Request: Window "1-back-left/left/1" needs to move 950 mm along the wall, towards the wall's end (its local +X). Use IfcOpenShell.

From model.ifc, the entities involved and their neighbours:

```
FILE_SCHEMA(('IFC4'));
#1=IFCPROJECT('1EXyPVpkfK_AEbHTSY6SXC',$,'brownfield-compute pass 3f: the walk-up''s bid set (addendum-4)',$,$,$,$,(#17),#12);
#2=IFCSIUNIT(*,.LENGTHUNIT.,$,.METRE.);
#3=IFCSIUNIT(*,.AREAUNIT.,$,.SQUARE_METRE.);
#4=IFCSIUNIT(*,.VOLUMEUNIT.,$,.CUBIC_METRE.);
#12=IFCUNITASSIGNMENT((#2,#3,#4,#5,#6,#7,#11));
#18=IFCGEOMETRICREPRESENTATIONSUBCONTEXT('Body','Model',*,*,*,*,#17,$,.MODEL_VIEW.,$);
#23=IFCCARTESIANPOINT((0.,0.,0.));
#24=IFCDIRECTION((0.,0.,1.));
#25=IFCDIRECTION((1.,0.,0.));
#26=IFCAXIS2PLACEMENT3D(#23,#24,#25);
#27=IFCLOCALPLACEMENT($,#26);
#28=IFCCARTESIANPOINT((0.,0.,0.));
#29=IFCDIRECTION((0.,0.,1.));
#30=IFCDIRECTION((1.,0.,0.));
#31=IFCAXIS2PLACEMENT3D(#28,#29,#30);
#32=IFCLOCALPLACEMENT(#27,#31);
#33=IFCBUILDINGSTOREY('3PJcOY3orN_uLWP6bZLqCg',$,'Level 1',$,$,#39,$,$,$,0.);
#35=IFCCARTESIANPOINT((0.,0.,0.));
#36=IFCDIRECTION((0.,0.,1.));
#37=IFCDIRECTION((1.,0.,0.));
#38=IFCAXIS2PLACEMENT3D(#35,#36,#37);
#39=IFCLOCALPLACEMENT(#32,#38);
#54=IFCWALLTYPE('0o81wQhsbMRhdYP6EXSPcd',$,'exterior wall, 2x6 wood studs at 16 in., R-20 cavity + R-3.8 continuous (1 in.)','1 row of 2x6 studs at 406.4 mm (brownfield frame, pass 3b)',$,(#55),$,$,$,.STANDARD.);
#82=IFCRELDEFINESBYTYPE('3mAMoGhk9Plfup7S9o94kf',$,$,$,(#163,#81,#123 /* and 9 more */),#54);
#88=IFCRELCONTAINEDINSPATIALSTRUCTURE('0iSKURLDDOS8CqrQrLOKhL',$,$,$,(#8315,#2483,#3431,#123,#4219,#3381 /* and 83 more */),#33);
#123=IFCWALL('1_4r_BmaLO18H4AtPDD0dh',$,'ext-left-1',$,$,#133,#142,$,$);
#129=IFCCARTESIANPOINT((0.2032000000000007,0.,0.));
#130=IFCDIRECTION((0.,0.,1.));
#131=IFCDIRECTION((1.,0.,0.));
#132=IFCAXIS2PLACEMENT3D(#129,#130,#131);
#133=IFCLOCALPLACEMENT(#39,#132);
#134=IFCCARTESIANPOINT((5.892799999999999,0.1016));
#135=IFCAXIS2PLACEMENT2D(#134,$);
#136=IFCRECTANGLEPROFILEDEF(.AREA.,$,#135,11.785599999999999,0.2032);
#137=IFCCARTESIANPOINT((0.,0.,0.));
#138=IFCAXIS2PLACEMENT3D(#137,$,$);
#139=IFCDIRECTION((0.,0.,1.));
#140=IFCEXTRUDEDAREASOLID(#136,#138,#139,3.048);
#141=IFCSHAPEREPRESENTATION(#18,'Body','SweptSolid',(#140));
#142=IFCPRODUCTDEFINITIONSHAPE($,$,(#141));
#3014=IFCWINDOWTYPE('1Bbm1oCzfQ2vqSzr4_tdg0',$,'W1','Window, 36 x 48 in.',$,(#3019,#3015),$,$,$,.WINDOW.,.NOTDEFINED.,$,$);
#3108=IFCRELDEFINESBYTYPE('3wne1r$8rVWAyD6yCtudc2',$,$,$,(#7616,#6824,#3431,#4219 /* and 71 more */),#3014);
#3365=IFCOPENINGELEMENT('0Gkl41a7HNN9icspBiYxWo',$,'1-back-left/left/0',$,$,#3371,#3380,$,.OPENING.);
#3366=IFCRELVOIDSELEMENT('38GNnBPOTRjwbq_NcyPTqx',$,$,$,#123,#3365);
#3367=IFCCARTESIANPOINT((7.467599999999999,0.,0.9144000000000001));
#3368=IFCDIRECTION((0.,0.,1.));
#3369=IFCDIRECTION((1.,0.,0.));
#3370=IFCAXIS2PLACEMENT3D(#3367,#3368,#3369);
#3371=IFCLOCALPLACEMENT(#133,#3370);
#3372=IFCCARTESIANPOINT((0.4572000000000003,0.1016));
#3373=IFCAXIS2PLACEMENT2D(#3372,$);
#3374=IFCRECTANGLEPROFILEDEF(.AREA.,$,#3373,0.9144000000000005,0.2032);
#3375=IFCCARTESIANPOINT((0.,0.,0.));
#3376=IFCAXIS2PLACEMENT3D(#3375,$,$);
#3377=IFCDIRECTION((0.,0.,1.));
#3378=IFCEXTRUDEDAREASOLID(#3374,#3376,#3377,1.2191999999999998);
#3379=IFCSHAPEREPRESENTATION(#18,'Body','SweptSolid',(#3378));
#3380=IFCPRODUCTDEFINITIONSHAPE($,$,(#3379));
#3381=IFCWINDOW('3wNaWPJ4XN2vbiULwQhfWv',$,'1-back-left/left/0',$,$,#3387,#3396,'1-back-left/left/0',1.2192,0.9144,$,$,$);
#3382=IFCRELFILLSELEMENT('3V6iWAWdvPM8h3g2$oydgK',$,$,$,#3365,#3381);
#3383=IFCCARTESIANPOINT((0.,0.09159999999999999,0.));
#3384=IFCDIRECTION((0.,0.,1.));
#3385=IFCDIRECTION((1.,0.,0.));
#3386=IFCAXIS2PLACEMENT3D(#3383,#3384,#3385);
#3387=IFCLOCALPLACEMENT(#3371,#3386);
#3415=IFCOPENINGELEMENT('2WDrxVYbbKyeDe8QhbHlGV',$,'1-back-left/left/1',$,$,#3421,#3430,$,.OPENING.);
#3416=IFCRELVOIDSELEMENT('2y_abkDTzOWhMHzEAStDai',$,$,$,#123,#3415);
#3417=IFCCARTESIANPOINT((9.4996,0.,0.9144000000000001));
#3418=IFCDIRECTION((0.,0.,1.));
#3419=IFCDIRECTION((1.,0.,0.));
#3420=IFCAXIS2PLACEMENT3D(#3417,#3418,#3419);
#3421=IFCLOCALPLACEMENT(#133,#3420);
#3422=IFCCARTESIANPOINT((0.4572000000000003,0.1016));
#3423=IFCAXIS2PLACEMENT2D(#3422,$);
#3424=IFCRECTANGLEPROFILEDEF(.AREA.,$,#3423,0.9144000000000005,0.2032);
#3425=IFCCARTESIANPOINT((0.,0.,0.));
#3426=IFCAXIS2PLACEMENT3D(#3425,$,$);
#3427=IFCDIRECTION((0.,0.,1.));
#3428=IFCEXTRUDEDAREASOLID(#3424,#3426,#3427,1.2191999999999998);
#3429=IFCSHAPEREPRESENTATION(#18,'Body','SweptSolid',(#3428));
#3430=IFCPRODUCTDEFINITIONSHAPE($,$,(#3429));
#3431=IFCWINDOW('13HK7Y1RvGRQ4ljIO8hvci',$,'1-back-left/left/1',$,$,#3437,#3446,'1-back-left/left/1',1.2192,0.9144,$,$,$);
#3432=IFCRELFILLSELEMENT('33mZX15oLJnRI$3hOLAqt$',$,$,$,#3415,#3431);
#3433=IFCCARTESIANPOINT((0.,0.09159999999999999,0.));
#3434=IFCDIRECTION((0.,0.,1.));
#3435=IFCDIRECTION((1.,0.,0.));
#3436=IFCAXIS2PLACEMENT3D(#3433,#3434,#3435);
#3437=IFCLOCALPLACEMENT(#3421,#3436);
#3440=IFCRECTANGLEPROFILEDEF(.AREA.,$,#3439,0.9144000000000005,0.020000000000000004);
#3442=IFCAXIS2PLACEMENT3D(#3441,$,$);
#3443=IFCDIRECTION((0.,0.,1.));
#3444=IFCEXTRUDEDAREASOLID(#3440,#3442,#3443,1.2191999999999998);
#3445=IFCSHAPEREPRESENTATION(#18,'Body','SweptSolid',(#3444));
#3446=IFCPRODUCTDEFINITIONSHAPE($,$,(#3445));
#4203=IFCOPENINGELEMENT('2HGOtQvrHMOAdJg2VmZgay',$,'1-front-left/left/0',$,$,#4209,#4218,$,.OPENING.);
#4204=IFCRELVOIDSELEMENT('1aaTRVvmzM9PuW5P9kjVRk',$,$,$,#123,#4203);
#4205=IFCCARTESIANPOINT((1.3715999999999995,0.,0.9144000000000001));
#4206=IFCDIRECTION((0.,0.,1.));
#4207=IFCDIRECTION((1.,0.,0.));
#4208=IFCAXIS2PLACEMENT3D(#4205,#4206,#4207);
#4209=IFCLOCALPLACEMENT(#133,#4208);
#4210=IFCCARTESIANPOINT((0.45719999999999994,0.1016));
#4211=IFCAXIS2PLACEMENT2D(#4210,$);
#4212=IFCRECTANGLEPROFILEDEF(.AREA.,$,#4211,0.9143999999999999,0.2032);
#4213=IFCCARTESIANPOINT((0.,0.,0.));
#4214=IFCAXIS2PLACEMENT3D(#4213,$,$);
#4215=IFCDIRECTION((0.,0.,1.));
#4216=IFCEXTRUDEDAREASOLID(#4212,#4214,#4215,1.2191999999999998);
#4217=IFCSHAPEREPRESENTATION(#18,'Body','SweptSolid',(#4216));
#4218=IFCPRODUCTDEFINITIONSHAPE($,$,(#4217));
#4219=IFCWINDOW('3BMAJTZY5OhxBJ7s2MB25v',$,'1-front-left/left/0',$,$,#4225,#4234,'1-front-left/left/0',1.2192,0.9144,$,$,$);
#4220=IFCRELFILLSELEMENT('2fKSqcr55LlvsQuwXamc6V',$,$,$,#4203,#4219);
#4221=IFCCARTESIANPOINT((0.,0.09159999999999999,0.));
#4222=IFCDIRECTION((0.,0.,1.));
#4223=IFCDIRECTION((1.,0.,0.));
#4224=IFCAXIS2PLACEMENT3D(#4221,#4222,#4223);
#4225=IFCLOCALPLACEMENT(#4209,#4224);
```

```python
import ifcopenshell
import ifcopenshell.api.geometry
import ifcopenshell.util.placement

model = ifcopenshell.open("model.ifc")

window = model.by_guid("13HK7Y1RvGRQ4ljIO8hvci")
opening = window.FillsVoids[0].RelatingOpeningElement
wall = opening.VoidsElements[0].RelatingBuildingElement

wall_matrix = ifcopenshell.util.placement.get_local_placement(wall.ObjectPlacement)
shift = wall_matrix[:3, 0] * 0.95
before = ifcopenshell.util.placement.get_local_placement(window.ObjectPlacement)[:3, 3].copy()

# The window is placed relative to its opening, so it follows when the opening moves.
matrix = ifcopenshell.util.placement.get_local_placement(opening.ObjectPlacement)
matrix[:3, 3] += shift
ifcopenshell.api.geometry.edit_object_placement(
    model, product=opening, matrix=matrix, is_si=False, should_transform_children=True
)

after = ifcopenshell.util.placement.get_local_placement(window.ObjectPlacement)[:3, 3]
print("window moved by", (after - before).round(3) + 0.0)

model.write("model_edited.ifc")
```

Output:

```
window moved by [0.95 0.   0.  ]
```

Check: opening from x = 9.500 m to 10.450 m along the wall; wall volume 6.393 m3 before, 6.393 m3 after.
